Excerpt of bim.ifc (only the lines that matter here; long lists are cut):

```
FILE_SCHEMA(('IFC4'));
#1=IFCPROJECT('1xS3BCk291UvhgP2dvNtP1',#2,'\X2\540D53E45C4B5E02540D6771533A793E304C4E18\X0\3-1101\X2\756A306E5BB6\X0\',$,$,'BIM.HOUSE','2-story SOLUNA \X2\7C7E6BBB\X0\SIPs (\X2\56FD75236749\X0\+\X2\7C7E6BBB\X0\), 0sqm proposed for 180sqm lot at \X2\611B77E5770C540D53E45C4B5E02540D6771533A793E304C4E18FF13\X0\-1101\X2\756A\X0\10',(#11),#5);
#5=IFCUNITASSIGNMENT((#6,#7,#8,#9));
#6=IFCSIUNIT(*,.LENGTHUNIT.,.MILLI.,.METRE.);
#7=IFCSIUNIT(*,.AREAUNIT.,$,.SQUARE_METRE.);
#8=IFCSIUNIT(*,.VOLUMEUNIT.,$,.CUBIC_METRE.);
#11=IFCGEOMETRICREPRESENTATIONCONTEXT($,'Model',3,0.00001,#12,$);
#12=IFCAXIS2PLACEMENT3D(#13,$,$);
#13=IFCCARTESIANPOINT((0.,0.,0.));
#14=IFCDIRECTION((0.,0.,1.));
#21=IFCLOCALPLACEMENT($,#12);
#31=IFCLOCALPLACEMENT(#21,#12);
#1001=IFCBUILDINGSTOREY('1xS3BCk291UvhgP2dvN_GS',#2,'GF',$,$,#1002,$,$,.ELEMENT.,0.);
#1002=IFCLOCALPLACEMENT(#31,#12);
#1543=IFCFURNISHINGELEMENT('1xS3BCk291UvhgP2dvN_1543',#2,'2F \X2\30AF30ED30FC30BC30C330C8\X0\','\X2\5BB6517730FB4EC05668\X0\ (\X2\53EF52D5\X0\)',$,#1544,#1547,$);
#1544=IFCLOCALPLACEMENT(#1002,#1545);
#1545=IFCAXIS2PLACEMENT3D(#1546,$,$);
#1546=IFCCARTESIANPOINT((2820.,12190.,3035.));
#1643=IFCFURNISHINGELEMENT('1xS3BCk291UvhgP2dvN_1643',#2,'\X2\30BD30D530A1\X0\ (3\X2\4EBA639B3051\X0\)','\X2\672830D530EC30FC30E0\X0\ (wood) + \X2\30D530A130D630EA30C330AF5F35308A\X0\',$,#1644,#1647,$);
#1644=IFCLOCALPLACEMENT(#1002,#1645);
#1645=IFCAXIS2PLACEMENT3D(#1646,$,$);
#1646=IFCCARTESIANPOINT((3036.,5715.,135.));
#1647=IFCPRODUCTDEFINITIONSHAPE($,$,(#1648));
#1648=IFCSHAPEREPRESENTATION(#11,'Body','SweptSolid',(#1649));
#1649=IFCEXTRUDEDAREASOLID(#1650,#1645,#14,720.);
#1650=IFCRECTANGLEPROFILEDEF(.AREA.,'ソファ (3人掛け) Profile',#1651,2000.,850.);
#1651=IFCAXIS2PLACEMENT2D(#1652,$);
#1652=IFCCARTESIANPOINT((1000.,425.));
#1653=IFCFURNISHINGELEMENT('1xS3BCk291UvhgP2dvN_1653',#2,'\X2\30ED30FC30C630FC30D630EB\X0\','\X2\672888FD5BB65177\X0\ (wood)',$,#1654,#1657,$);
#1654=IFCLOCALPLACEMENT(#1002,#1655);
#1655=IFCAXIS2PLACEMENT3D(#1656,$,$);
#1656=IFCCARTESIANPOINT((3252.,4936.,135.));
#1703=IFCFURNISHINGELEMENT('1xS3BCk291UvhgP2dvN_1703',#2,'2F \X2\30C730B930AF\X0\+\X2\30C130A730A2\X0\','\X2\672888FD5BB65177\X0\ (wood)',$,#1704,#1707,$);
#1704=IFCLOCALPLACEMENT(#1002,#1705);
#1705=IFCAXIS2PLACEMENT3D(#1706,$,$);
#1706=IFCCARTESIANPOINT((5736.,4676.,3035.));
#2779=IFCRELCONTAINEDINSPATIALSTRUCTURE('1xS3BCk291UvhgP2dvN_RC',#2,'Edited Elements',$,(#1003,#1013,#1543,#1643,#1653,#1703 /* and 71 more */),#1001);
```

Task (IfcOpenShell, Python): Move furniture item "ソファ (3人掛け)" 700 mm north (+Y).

```python
import ifcopenshell
import ifcopenshell.api.geometry
import ifcopenshell.util.placement

model = ifcopenshell.open("bim.ifc")

item = model.by_guid("1xS3BCk291UvhgP2dvN_1643")
matrix = ifcopenshell.util.placement.get_local_placement(item.ObjectPlacement)
matrix[1, 3] += 700.0
ifcopenshell.api.geometry.edit_object_placement(model, product=item, matrix=matrix, is_si=False)

print(ifcopenshell.util.placement.get_local_placement(item.ObjectPlacement).round(3) + 0.0)

model.write("bim_edited.ifc")
```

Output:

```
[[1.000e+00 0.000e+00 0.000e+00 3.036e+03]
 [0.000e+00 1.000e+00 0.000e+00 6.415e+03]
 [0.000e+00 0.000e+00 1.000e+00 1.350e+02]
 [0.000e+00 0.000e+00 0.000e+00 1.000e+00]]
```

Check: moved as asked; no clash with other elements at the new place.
